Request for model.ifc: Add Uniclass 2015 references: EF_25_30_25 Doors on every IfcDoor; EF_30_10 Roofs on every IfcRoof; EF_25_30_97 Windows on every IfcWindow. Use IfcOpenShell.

First a look at what the model holds.

```python
import ifcopenshell

model = ifcopenshell.open("model.ifc")
print(model.schema)
print("classifications:", [c.Name for c in model.by_type("IfcClassification")])
for ifc_class in ("IfcDoor", "IfcRoof", "IfcStair", "IfcWall", "IfcWindow"):
    print(ifc_class, len(model.by_type(ifc_class)))
```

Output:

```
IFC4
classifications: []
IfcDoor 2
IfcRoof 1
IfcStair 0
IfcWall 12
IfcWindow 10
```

```python
import ifcopenshell
import ifcopenshell.api.classification

model = ifcopenshell.open("model.ifc")

system = ifcopenshell.api.classification.add_classification(model, classification="Uniclass 2015")

codes = {
    "IfcDoor": ("EF_25_30_25", "Doors"),
    "IfcRoof": ("EF_30_10", "Roofs"),
    "IfcWindow": ("EF_25_30_97", "Windows"),
}
for ifc_class, (code, name) in codes.items():
    products = model.by_type(ifc_class)
    ifcopenshell.api.classification.add_reference(
        model, products=products, classification=system, identification=code, name=name
    )
    print(code, len(products))

model.write("model_v2.ifc")
```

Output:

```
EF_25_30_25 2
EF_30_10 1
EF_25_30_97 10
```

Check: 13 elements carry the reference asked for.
